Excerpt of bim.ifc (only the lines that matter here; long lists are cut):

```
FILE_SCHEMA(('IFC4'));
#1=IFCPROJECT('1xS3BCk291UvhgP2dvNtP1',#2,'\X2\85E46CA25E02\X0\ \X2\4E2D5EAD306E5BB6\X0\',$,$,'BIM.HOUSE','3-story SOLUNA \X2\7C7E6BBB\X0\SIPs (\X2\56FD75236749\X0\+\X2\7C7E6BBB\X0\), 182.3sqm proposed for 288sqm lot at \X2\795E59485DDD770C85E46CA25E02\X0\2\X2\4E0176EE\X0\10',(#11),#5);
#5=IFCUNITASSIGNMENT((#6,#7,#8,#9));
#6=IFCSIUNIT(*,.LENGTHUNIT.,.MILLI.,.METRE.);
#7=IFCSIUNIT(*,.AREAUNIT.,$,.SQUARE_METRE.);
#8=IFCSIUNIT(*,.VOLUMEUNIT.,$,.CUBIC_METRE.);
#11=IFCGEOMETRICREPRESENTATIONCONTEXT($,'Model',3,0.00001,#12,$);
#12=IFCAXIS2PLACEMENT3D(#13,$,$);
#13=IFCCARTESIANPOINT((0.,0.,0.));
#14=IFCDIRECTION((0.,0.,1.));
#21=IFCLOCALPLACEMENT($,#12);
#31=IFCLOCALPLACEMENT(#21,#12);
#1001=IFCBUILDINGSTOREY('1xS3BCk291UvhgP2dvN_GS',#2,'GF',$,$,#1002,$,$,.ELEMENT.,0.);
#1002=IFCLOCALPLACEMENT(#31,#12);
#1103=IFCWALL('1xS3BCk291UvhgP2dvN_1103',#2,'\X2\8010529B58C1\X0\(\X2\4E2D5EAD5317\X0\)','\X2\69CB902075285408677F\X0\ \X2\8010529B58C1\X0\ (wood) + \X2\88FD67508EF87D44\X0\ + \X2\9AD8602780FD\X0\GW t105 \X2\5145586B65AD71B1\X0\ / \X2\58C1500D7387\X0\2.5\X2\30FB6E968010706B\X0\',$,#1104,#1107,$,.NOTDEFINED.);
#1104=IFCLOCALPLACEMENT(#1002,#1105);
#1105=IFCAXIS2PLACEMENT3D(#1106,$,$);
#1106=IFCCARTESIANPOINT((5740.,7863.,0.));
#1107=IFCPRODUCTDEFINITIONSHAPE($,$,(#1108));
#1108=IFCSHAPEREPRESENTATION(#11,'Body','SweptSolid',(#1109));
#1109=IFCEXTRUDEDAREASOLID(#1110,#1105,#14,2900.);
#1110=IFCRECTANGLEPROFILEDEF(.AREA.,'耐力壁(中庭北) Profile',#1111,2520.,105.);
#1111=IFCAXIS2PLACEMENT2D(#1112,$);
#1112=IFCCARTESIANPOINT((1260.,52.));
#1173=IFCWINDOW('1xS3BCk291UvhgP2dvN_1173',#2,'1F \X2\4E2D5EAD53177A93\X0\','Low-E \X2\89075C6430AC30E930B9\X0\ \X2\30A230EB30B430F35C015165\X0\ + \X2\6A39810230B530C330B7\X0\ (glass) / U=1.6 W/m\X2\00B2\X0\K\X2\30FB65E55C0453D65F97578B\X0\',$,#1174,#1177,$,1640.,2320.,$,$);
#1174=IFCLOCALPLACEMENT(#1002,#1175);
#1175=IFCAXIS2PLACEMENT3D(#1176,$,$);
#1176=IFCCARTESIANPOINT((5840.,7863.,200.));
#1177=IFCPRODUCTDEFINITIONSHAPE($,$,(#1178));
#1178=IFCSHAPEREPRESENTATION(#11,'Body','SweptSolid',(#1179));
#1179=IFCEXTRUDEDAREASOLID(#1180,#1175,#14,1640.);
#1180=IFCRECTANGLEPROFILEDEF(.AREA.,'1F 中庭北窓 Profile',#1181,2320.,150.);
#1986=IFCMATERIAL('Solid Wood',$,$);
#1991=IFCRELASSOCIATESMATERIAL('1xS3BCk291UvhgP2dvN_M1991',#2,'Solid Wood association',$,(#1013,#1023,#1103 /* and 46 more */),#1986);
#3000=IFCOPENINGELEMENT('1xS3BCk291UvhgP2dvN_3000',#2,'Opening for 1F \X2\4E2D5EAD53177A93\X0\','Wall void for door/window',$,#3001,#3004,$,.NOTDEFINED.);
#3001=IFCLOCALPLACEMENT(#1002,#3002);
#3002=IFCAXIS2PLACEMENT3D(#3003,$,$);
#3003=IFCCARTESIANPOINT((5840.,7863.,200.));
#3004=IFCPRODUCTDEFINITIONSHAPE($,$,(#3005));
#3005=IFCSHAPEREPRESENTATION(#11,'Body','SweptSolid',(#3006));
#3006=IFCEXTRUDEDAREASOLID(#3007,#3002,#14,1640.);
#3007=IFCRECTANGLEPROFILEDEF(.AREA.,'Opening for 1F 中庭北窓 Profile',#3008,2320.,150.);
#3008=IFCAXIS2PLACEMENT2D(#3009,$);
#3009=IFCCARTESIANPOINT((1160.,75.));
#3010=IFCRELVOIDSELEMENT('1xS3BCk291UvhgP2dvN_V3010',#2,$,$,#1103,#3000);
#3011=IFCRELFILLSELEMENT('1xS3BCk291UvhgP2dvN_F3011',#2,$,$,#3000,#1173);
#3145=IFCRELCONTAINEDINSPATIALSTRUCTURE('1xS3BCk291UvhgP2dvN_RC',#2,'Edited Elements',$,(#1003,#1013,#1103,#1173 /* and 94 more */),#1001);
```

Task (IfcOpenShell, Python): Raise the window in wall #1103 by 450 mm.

```python
import numpy as np
import ifcopenshell
import ifcopenshell.api.geometry
import ifcopenshell.util.placement
import ifcopenshell.util.unit

model = ifcopenshell.open("bim.ifc")
unit_scale = ifcopenshell.util.unit.calculate_unit_scale(model)

window = model.by_guid("1xS3BCk291UvhgP2dvN_1173")
opening = window.FillsVoids[0].RelatingOpeningElement
dz = 0.45 / unit_scale

shift = np.array([0.0, 0.0, dz])
# The window is not placed relative to its opening, so move both.
for product in (opening, window):
    matrix = ifcopenshell.util.placement.get_local_placement(product.ObjectPlacement)
    matrix[:3, 3] += shift
    ifcopenshell.api.geometry.edit_object_placement(model, product=product, matrix=matrix, is_si=False)

print(f"moved by {dz * unit_scale:+.3f} m")

model.write("bim_rev.ifc")
```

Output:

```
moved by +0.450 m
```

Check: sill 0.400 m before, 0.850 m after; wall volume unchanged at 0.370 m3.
